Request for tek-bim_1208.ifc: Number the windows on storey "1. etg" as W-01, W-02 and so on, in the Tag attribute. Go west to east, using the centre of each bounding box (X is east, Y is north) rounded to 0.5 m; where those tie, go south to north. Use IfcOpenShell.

First a look at what the model holds.

```python
import ifcopenshell
import ifcopenshell.util.element
import ifcopenshell.util.placement

model = ifcopenshell.open("tek-bim_1208.ifc")
print(model.schema)
storey = next(s for s in model.by_type("IfcBuildingStorey") if s.Name == "1. etg")
windows = [e for e in ifcopenshell.util.element.get_decomposition(storey) if e.is_a("IfcWindow")]
for e in sorted(windows, key=lambda e: e.id()):
    origin = ifcopenshell.util.placement.get_local_placement(e.ObjectPlacement)[:3, 3]
    print(e.id(), e.Tag, e.Name, origin.round(2) + 0.0, sep=" | ")
```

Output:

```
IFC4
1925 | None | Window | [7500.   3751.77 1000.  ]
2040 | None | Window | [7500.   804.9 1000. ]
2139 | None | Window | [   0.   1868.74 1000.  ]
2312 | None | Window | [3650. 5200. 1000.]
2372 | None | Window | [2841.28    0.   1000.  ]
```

```python
import ifcopenshell
import ifcopenshell.geom
import ifcopenshell.util.element
import ifcopenshell.util.shape

model = ifcopenshell.open("tek-bim_1208.ifc")
settings = ifcopenshell.geom.settings()
settings.set("use-world-coords", True)


def centre(element):
    shape = ifcopenshell.geom.create_shape(settings, element)
    return ifcopenshell.util.shape.get_bbox_centroid(shape.geometry)


storey = next(s for s in model.by_type("IfcBuildingStorey") if s.Name == "1. etg")
windows = [e for e in ifcopenshell.util.element.get_decomposition(storey) if e.is_a("IfcWindow")]

# Insertion points can sit at a corner or the storey origin, so sort by the geometry (in metres).
centres = {e: centre(e) for e in windows}
windows.sort(key=lambda e: (round(centres[e][0] / 0.5), centres[e][1]))

for i, e in enumerate(windows, start=1):
    number = f"W-{i:02d}"
    e.Tag = number
    print(e.id(), number)

model.write("tek-bim_1208-out.ifc")
```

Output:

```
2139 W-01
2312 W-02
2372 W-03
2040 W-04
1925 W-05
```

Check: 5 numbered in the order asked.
